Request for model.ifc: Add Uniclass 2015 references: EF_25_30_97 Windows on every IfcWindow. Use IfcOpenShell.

First a look at what the model holds.

```python
import ifcopenshell

model = ifcopenshell.open("model.ifc")
print(model.schema)
print("classifications:", [c.Name for c in model.by_type("IfcClassification")])
for ifc_class in ("IfcDoor", "IfcRoof", "IfcStair", "IfcWall", "IfcWindow"):
    print(ifc_class, len(model.by_type(ifc_class)))
```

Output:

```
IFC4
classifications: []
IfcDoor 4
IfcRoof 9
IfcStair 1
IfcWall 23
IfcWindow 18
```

```python
import ifcopenshell
import ifcopenshell.api.classification

model = ifcopenshell.open("model.ifc")

system = ifcopenshell.api.classification.add_classification(model, classification="Uniclass 2015")

codes = {
    "IfcWindow": ("EF_25_30_97", "Windows"),
}
for ifc_class, (code, name) in codes.items():
    products = model.by_type(ifc_class)
    ifcopenshell.api.classification.add_reference(
        model, products=products, classification=system, identification=code, name=name
    )
    print(code, len(products))

model.write("model_v2.ifc")
```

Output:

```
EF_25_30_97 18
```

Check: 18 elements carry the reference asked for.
